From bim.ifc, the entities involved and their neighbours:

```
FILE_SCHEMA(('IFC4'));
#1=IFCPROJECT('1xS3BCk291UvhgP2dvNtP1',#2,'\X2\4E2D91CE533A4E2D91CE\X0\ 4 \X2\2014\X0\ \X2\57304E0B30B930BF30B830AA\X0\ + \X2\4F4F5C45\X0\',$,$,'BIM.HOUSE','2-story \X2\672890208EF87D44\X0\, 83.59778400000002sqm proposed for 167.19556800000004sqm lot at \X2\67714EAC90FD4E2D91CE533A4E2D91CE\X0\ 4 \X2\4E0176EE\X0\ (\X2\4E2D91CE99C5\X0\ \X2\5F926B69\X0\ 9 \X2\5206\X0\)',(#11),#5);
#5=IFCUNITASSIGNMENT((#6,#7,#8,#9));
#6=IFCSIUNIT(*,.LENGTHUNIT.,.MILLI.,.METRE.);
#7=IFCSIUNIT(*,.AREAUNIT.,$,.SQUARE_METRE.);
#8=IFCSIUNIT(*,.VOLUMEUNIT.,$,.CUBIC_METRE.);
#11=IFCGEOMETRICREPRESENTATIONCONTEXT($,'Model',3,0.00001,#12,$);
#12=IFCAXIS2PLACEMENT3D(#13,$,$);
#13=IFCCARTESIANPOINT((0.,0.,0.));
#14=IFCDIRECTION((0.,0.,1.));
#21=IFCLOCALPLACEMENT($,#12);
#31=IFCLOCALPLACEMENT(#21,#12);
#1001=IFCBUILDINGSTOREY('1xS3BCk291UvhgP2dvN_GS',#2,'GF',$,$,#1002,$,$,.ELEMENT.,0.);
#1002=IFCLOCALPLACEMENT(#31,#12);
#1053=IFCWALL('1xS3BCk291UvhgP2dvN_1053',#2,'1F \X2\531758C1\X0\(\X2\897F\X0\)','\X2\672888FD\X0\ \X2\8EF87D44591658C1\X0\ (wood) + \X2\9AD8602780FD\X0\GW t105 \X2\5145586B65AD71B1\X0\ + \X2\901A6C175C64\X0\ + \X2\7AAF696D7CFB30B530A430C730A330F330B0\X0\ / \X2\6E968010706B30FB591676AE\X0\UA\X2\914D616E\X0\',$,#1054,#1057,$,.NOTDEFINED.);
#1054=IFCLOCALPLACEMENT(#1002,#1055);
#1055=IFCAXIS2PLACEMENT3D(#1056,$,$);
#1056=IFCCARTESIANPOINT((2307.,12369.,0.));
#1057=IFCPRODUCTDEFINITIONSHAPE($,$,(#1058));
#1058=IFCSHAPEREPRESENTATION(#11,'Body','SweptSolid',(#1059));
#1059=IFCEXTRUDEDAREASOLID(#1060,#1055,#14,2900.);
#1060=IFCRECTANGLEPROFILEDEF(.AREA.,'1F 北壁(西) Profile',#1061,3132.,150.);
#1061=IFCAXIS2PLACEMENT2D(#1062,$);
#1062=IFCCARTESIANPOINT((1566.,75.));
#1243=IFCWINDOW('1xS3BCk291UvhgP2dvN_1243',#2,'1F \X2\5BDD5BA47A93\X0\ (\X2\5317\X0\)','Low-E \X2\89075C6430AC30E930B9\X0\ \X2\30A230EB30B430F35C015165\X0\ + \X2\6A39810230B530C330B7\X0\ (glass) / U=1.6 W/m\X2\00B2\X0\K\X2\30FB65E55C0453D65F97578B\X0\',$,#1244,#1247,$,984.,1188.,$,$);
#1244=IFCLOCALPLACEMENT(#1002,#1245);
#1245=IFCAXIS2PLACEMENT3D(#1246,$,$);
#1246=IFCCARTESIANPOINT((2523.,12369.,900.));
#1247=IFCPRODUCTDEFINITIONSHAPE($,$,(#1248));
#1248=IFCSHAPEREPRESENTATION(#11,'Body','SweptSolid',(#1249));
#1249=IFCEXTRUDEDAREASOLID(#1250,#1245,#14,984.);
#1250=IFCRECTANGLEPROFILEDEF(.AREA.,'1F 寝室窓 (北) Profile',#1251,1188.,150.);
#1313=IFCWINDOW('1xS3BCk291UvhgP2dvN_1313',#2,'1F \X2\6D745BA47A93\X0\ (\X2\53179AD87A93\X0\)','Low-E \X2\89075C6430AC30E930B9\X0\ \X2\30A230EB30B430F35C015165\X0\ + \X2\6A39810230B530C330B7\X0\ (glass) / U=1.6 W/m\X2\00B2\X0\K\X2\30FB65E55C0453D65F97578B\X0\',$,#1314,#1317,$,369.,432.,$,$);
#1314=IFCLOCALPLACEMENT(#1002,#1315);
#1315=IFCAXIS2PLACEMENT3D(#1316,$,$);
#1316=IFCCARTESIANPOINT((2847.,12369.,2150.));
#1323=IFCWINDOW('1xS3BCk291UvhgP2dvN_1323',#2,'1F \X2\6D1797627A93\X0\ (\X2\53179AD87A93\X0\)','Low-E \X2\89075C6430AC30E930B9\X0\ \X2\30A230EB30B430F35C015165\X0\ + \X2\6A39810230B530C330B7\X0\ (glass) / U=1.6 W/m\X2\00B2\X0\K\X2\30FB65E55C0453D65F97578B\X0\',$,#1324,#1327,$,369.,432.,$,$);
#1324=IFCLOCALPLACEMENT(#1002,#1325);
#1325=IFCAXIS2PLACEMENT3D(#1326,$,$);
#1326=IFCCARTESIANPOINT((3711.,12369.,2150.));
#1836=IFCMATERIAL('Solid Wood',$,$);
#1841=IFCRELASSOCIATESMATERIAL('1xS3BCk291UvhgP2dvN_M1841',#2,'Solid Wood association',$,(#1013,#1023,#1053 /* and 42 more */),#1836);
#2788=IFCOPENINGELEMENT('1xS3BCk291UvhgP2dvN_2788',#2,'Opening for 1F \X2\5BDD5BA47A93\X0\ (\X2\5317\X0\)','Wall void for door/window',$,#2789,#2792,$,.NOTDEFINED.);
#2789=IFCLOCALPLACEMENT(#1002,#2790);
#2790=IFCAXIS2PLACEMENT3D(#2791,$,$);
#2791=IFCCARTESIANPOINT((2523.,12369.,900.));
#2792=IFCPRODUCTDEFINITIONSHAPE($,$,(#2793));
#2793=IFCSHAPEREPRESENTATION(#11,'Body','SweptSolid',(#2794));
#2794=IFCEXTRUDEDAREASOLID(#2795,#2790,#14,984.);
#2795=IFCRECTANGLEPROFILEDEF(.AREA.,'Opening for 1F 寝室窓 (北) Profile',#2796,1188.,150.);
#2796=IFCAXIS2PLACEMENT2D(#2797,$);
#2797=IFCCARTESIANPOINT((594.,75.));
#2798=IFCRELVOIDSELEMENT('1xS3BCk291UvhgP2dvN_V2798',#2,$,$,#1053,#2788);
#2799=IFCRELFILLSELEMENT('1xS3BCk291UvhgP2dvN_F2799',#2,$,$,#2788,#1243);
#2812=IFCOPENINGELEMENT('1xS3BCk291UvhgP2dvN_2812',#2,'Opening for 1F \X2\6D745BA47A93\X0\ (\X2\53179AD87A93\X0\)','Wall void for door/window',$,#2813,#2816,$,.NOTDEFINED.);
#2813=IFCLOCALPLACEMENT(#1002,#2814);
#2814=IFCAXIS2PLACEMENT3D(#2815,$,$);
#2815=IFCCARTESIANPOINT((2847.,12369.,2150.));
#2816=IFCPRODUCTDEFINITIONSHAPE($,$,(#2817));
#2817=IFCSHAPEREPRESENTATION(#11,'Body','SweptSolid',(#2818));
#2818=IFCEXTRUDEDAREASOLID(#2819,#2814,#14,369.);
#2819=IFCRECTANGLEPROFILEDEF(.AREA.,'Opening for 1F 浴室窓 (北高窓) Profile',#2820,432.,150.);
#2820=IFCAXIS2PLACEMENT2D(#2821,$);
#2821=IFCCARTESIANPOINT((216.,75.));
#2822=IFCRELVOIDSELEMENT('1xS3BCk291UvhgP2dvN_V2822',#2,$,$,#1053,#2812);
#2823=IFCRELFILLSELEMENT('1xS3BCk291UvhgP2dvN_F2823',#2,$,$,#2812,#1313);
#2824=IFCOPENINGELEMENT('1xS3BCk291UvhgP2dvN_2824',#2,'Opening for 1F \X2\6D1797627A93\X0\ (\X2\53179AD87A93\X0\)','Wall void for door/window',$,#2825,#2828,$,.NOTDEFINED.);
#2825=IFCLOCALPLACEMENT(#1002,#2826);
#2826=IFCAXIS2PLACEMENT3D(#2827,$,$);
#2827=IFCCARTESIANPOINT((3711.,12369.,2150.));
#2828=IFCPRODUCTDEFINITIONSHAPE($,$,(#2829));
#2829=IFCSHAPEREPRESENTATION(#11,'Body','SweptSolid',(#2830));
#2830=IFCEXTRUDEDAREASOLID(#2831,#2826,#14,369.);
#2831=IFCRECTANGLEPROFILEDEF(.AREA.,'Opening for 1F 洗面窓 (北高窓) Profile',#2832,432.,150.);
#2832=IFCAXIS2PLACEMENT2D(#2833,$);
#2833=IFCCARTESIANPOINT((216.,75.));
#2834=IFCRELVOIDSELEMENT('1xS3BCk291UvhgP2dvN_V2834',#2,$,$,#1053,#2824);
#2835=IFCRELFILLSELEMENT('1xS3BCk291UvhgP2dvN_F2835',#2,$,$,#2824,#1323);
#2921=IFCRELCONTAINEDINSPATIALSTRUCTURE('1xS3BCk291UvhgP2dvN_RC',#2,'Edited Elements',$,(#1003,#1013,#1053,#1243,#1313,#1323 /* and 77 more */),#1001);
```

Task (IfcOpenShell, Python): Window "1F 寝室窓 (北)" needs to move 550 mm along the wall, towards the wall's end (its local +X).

```python
import ifcopenshell
import ifcopenshell.api.geometry
import ifcopenshell.util.placement
import ifcopenshell.util.unit

model = ifcopenshell.open("bim.ifc")
unit_scale = ifcopenshell.util.unit.calculate_unit_scale(model)

window = model.by_guid("1xS3BCk291UvhgP2dvN_1243")
opening = window.FillsVoids[0].RelatingOpeningElement
wall = opening.VoidsElements[0].RelatingBuildingElement

wall_matrix = ifcopenshell.util.placement.get_local_placement(wall.ObjectPlacement)
shift = wall_matrix[:3, 0] * 0.55 / unit_scale
before = ifcopenshell.util.placement.get_local_placement(window.ObjectPlacement)[:3, 3].copy()

# The window is not placed relative to its opening, so move both.
for product in (opening, window):
    matrix = ifcopenshell.util.placement.get_local_placement(product.ObjectPlacement)
    matrix[:3, 3] += shift
    ifcopenshell.api.geometry.edit_object_placement(model, product=product, matrix=matrix, is_si=False)

after = ifcopenshell.util.placement.get_local_placement(window.ObjectPlacement)[:3, 3]
print("window moved by", (after - before).round(3) + 0.0)

model.write("bim_rev.ifc")
```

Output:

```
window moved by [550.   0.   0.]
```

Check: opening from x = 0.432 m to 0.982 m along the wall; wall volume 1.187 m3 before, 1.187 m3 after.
